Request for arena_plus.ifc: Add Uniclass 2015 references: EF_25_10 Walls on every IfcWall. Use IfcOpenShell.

First a look at what the model holds.

```python
import ifcopenshell

model = ifcopenshell.open("arena_plus.ifc")
print(model.schema)
print("classifications:", [c.Name for c in model.by_type("IfcClassification")])
for ifc_class in ("IfcDoor", "IfcRoof", "IfcStair", "IfcWall", "IfcWindow"):
    print(ifc_class, len(model.by_type(ifc_class)))
```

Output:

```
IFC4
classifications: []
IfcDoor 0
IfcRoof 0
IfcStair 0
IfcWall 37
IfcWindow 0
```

```python
import ifcopenshell
import ifcopenshell.api.classification

model = ifcopenshell.open("arena_plus.ifc")

system = ifcopenshell.api.classification.add_classification(model, classification="Uniclass 2015")

codes = {
    "IfcWall": ("EF_25_10", "Walls"),
}
for ifc_class, (code, name) in codes.items():
    products = model.by_type(ifc_class)
    ifcopenshell.api.classification.add_reference(
        model, products=products, classification=system, identification=code, name=name
    )
    print(code, len(products))

model.write("arena_plus_rev.ifc")
```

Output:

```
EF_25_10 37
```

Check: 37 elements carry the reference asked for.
